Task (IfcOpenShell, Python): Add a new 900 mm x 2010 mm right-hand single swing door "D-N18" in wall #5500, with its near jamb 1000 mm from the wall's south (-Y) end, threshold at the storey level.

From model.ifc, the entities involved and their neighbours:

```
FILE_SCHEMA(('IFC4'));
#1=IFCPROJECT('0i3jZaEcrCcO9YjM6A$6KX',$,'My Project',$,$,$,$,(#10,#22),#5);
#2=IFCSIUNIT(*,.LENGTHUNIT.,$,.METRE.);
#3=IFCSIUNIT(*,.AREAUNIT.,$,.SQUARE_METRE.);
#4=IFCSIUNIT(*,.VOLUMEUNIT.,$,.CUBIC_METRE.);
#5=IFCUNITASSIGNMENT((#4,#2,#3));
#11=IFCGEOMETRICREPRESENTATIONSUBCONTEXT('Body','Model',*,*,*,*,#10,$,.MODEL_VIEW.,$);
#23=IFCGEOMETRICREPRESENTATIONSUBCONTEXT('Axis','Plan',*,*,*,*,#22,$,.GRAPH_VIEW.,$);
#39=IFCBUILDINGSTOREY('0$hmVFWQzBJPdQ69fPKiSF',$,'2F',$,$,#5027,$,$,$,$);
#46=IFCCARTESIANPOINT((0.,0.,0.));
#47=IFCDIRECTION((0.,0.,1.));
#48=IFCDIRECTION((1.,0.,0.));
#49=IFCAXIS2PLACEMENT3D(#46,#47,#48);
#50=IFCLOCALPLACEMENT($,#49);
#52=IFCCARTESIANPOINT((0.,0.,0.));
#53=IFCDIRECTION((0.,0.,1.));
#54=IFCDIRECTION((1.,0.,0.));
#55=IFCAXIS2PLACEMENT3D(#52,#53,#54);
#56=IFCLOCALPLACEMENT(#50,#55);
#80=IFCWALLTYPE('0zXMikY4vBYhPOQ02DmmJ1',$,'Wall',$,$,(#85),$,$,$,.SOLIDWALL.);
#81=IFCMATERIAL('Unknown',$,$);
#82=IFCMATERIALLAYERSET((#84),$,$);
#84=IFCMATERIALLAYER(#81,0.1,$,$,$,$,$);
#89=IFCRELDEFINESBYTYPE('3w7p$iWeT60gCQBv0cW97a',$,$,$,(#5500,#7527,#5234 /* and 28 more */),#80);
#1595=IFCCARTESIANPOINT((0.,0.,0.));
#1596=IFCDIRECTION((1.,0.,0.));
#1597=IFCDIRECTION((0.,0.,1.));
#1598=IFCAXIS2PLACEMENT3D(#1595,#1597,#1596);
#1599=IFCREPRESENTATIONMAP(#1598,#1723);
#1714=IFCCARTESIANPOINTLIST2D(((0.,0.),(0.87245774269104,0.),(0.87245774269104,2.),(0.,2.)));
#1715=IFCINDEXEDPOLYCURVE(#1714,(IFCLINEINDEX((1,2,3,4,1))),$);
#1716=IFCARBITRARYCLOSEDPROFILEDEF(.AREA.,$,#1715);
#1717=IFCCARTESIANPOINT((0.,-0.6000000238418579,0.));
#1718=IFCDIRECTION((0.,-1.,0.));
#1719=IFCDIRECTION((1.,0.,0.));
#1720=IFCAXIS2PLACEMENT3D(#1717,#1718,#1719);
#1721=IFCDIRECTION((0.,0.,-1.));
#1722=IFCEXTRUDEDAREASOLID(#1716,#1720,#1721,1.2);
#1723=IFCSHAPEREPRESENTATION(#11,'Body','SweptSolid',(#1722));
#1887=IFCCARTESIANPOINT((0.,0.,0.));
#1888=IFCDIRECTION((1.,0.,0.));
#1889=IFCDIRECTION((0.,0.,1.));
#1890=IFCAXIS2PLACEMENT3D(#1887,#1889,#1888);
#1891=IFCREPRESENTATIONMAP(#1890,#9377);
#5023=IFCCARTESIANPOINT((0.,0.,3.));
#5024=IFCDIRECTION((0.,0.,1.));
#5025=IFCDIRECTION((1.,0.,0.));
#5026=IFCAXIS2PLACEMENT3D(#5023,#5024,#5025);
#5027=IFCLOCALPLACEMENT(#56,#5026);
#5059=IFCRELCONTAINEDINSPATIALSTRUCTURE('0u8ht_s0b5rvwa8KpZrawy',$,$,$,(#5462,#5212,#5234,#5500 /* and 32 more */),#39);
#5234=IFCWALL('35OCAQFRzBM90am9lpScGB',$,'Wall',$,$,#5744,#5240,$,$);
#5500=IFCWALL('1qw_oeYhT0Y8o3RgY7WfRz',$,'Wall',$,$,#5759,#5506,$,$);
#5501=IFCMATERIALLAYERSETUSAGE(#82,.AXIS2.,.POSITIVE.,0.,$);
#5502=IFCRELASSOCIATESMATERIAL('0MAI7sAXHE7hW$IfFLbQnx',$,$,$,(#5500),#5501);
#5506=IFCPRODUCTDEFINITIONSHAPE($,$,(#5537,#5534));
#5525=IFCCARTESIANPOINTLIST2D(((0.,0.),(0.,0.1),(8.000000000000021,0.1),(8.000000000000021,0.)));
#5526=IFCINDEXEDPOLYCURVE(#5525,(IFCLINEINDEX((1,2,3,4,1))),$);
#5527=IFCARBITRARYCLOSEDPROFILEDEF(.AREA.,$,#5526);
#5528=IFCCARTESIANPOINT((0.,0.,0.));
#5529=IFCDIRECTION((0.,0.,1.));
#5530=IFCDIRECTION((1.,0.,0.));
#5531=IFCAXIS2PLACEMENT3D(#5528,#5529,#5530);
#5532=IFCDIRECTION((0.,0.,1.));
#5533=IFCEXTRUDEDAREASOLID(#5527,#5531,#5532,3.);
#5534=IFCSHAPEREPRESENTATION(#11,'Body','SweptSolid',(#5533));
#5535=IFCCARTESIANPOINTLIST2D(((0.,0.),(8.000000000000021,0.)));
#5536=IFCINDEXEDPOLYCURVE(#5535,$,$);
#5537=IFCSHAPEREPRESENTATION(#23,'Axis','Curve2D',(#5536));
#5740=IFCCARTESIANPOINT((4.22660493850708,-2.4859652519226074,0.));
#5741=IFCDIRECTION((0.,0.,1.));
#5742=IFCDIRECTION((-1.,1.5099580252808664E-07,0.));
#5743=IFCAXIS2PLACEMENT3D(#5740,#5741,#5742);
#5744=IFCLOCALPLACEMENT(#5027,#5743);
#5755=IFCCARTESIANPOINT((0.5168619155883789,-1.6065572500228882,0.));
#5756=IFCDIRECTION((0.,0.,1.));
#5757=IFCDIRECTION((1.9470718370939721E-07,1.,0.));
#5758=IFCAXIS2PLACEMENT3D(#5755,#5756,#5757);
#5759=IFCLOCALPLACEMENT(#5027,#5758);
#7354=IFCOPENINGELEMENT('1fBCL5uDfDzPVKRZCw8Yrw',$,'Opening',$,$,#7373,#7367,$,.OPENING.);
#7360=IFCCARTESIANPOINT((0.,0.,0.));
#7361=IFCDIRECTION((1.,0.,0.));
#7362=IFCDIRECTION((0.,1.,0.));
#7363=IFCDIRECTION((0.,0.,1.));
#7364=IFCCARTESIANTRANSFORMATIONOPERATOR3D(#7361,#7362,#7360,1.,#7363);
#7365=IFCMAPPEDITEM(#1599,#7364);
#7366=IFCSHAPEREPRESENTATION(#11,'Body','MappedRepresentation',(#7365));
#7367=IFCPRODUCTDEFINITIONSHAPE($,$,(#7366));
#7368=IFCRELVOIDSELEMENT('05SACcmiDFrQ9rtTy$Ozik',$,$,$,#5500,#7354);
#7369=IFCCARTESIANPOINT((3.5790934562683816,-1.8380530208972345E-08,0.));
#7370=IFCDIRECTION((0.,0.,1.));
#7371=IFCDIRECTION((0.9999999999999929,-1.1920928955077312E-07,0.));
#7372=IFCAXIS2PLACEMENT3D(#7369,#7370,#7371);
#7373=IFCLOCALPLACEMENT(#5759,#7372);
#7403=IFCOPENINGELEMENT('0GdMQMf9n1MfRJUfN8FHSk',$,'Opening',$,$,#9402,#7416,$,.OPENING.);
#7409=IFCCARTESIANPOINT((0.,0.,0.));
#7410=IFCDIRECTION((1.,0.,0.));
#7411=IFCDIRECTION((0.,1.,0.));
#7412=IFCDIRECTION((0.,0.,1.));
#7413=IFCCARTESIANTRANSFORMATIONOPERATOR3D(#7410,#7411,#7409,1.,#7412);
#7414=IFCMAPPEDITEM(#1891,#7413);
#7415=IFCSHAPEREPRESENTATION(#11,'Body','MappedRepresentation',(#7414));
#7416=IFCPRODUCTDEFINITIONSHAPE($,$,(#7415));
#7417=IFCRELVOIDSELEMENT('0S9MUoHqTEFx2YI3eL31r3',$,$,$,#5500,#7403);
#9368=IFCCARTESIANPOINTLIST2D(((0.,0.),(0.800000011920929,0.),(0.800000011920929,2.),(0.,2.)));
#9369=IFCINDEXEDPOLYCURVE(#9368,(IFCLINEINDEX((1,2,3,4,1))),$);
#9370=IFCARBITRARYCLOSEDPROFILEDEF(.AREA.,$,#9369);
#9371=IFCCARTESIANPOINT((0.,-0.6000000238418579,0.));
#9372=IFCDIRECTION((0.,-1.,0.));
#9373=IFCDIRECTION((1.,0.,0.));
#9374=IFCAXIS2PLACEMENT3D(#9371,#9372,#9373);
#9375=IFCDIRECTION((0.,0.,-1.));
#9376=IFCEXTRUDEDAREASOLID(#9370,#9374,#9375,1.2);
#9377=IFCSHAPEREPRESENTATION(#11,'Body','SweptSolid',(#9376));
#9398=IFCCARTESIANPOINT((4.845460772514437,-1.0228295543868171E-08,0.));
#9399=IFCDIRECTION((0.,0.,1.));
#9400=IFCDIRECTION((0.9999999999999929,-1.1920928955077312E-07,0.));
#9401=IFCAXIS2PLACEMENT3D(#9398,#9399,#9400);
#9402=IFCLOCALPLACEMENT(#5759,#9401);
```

```python
import numpy as np
import ifcopenshell
import ifcopenshell.api.feature
import ifcopenshell.api.geometry
import ifcopenshell.api.root
import ifcopenshell.api.spatial
import ifcopenshell.geom
import ifcopenshell.util.element
import ifcopenshell.util.placement
import ifcopenshell.util.representation
import ifcopenshell.util.shape
import ifcopenshell.util.unit

model = ifcopenshell.open("model.ifc")
unit_scale = ifcopenshell.util.unit.calculate_unit_scale(model)
settings = ifcopenshell.geom.settings()


def volume(element):
    """Net volume in cubic metres, openings subtracted."""
    shape = ifcopenshell.geom.create_shape(settings, element)
    return ifcopenshell.util.shape.get_volume(shape.geometry)


wall = model.by_id(5500)
storey = ifcopenshell.util.element.get_container(wall, ifc_class="IfcBuildingStorey")
context = ifcopenshell.util.representation.get_context(model, "Model", "Body", "MODEL_VIEW")
before = volume(wall)

width, height, from_end, sill = 0.9, 2.01, 1, 0.0  # metres

# The wall runs along its own X axis, and the end named is its -X end.
wall_shape = ifcopenshell.geom.create_shape(settings, wall)
x, y, z = ifcopenshell.util.shape.get_vertices(wall_shape.geometry).T
start = x.min() + from_end
face, thickness = float(y.min()), float(y.max() - y.min())
wall_matrix = ifcopenshell.util.placement.get_local_placement(wall.ObjectPlacement)
level = ifcopenshell.util.placement.get_local_placement(storey.ObjectPlacement)[2, 3]


def in_wall(x, y):
    """Placement at x, y metres in the wall's axes, at sill height."""
    matrix = wall_matrix.copy()
    matrix[:, 3] = wall_matrix @ np.array([x / unit_scale, y / unit_scale, 0.0, 1.0])
    matrix[2, 3] = level + sill / unit_scale
    return matrix


# Opening: a box that overshoots both wall faces by 50 mm.
opening = ifcopenshell.api.root.create_entity(model, ifc_class="IfcOpeningElement", predefined_type="OPENING")
box = ifcopenshell.api.geometry.add_wall_representation(
    model, context=context, length=width, height=height, thickness=thickness + 0.1
)
ifcopenshell.api.geometry.assign_representation(model, product=opening, representation=box)
ifcopenshell.api.geometry.edit_object_placement(model, product=opening, matrix=in_wall(start, face - 0.05), is_si=False)
ifcopenshell.api.feature.add_feature(model, feature=opening, element=wall)

door = ifcopenshell.api.root.create_entity(model, ifc_class="IfcDoor", name="D-N18", predefined_type="DOOR")
door.OverallWidth, door.OverallHeight = width / unit_scale, height / unit_scale
door.OperationType = "SINGLE_SWING_RIGHT"
body = ifcopenshell.api.geometry.add_door_representation(
    model,
    context=context,
    overall_width=door.OverallWidth,
    overall_height=door.OverallHeight,
    operation_type="SINGLE_SWING_RIGHT",
    lining_properties={"LiningDepth": thickness / unit_scale, "ThresholdDepth": thickness / unit_scale},
)
ifcopenshell.api.geometry.assign_representation(model, product=door, representation=body)
ifcopenshell.api.spatial.assign_container(model, products=[door], relating_structure=storey)
ifcopenshell.api.feature.add_filling(model, opening=opening, element=door)

# The lining spans the wall, so the door starts at the wall face.
ifcopenshell.api.geometry.edit_object_placement(model, product=door, matrix=in_wall(start, face), is_si=False)

after = volume(wall)

print(f"wall volume {before:.3f} -> {after:.3f} m3")

model.write("model_v2.ifc")
```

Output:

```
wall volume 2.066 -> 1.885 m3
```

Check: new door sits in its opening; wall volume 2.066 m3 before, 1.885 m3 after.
